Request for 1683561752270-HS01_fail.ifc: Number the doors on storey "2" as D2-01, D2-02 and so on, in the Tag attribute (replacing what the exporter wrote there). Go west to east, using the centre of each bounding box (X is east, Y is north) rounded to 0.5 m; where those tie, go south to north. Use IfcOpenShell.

First a look at what the model holds.

```python
import ifcopenshell
import ifcopenshell.util.element
import ifcopenshell.util.placement

model = ifcopenshell.open("1683561752270-HS01_fail.ifc")
print(model.schema)
storey = next(s for s in model.by_type("IfcBuildingStorey") if s.Name == "2")
doors = [e for e in ifcopenshell.util.element.get_decomposition(storey) if e.is_a("IfcDoor")]
for e in sorted(doors, key=lambda e: e.id()):
    origin = ifcopenshell.util.placement.get_local_placement(e.ObjectPlacement)[:3, 3]
    print(e.id(), e.Tag, e.Name, origin.round(2) + 0.0, sep=" | ")
```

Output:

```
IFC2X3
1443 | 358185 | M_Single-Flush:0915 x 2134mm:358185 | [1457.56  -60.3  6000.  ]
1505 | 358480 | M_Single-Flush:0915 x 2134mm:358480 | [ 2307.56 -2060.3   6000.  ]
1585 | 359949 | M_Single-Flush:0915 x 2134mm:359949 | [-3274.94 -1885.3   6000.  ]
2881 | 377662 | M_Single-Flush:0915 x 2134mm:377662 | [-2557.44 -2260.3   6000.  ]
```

```python
import ifcopenshell
import ifcopenshell.geom
import ifcopenshell.util.element
import ifcopenshell.util.shape

model = ifcopenshell.open("1683561752270-HS01_fail.ifc")
settings = ifcopenshell.geom.settings()
settings.set("use-world-coords", True)


def centre(element):
    shape = ifcopenshell.geom.create_shape(settings, element)
    return ifcopenshell.util.shape.get_bbox_centroid(shape.geometry)


storey = next(s for s in model.by_type("IfcBuildingStorey") if s.Name == "2")
doors = [e for e in ifcopenshell.util.element.get_decomposition(storey) if e.is_a("IfcDoor")]

# Insertion points can sit at a corner or the storey origin, so sort by the geometry (in metres).
centres = {e: centre(e) for e in doors}
doors.sort(key=lambda e: (round(centres[e][0] / 0.5), centres[e][1]))

for i, e in enumerate(doors, start=1):
    number = f"D2-{i:02d}"
    e.Tag = number
    print(e.id(), number)

model.write("1683561752270-HS01_fail-out.ifc")
```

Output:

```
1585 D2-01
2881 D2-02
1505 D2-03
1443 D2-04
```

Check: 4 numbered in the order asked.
